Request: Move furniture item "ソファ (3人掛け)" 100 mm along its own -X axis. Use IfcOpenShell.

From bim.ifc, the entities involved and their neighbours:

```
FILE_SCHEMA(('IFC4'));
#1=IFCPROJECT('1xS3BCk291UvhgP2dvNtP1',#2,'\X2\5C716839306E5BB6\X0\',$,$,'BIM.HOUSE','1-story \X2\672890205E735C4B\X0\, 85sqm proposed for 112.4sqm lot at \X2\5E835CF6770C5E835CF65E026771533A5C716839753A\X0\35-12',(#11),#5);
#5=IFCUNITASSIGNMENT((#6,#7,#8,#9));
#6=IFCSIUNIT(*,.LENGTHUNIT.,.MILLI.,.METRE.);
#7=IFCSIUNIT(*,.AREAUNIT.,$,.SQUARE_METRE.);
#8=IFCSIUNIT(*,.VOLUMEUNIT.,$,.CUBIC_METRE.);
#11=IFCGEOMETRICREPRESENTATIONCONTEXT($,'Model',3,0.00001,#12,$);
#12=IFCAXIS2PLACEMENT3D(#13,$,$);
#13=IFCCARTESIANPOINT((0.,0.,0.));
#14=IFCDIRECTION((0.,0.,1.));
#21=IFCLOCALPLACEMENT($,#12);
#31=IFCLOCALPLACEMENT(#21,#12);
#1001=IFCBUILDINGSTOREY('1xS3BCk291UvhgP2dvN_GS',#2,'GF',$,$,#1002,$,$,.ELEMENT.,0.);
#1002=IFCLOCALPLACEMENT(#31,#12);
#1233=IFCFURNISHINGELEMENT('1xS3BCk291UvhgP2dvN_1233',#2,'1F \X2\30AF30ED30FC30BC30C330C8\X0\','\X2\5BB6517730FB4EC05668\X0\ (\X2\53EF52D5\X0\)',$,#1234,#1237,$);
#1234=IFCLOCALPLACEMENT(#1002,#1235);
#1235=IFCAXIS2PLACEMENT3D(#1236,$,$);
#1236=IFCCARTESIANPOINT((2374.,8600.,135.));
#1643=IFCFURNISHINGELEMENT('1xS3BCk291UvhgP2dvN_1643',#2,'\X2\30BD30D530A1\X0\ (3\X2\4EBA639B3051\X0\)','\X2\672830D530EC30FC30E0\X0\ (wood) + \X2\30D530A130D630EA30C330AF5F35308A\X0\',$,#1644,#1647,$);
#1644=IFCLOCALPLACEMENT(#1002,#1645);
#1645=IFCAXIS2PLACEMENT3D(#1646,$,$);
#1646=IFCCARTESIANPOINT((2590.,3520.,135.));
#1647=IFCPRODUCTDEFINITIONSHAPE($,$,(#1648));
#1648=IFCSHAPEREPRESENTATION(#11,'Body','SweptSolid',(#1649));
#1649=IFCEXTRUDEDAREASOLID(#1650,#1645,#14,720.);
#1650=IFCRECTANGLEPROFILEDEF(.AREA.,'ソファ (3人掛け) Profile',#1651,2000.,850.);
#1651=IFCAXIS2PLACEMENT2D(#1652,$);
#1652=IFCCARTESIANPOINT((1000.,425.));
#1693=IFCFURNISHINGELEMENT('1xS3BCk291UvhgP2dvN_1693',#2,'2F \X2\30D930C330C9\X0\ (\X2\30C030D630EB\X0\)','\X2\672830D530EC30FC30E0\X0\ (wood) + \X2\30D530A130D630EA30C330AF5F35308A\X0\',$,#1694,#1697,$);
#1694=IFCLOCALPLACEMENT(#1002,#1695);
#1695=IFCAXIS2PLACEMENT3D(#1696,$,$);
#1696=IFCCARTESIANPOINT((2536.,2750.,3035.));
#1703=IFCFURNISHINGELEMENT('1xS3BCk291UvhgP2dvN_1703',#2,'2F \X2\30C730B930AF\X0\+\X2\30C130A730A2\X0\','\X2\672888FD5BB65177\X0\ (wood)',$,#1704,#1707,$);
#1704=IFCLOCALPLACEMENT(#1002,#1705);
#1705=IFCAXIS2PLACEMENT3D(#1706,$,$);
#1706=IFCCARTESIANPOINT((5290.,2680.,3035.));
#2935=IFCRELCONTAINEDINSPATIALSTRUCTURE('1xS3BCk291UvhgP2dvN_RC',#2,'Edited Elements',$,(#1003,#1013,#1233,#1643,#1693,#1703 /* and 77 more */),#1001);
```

```python
import ifcopenshell
import ifcopenshell.api.geometry
import ifcopenshell.util.placement
import ifcopenshell.util.unit

model = ifcopenshell.open("bim.ifc")
unit_scale = ifcopenshell.util.unit.calculate_unit_scale(model)

item = model.by_guid("1xS3BCk291UvhgP2dvN_1643")
matrix = ifcopenshell.util.placement.get_local_placement(item.ObjectPlacement)
matrix[:3, 3] -= matrix[:3, 0] * 0.1 / unit_scale
ifcopenshell.api.geometry.edit_object_placement(model, product=item, matrix=matrix, is_si=False)

print(ifcopenshell.util.placement.get_local_placement(item.ObjectPlacement).round(3) + 0.0)

model.write("bim_edited.ifc")
```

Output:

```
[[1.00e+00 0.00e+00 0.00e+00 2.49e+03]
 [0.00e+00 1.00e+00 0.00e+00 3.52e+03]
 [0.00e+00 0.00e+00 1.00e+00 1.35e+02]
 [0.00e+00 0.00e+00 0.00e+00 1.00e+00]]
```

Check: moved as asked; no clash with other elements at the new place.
